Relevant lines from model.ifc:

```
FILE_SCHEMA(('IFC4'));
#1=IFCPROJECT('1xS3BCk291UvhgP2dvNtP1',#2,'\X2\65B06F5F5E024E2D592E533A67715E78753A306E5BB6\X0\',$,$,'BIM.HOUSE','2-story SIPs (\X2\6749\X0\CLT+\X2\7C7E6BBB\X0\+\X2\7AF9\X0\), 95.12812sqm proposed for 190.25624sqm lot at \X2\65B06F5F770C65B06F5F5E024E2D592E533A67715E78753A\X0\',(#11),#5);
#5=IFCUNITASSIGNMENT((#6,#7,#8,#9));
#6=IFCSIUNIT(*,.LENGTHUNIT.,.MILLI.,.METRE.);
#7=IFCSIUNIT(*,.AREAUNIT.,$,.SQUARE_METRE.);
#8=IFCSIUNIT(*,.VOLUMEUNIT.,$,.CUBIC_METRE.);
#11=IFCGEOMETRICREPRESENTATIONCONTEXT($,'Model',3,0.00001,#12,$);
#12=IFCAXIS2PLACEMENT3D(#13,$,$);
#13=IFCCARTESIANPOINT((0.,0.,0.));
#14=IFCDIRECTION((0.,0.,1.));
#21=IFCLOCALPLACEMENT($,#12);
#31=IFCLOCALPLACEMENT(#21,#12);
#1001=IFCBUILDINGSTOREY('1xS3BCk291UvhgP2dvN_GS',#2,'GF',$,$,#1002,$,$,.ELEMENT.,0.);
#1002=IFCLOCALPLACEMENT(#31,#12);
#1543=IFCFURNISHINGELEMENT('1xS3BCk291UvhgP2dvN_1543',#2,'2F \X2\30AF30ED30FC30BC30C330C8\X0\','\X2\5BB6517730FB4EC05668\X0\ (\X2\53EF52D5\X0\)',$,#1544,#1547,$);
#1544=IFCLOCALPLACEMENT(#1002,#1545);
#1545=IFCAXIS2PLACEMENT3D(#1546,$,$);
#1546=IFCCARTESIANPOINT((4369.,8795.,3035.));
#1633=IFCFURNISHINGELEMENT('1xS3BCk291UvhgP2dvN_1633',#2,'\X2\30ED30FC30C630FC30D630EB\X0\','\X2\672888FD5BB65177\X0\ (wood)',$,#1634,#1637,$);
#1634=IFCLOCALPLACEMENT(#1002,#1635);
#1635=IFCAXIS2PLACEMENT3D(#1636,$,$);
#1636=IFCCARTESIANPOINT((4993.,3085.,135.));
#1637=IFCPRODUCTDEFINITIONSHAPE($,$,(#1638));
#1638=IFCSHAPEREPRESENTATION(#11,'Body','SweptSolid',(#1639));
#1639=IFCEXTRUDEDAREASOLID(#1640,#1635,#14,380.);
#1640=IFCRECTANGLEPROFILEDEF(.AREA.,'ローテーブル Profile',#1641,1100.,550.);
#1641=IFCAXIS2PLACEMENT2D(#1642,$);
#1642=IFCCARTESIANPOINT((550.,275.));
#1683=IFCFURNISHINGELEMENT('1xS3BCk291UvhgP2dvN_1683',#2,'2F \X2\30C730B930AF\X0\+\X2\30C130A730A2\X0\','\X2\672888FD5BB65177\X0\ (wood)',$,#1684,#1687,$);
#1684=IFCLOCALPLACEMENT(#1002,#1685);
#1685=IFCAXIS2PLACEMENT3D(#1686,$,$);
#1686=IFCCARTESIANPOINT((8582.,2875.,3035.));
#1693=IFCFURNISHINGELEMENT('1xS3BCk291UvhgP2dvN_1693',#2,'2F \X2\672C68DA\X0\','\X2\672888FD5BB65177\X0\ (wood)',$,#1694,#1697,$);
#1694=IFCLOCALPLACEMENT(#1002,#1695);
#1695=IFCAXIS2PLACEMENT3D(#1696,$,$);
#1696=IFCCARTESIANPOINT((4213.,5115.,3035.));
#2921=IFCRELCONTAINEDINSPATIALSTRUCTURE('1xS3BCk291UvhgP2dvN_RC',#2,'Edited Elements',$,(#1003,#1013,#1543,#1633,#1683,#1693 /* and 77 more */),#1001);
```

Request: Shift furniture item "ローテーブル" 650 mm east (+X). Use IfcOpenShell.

```python
import ifcopenshell
import ifcopenshell.api.geometry
import ifcopenshell.util.placement

model = ifcopenshell.open("model.ifc")

item = model.by_guid("1xS3BCk291UvhgP2dvN_1633")
matrix = ifcopenshell.util.placement.get_local_placement(item.ObjectPlacement)
matrix[0, 3] += 650.0
ifcopenshell.api.geometry.edit_object_placement(model, product=item, matrix=matrix, is_si=False)

print(ifcopenshell.util.placement.get_local_placement(item.ObjectPlacement).round(3) + 0.0)

model.write("model-out.ifc")
```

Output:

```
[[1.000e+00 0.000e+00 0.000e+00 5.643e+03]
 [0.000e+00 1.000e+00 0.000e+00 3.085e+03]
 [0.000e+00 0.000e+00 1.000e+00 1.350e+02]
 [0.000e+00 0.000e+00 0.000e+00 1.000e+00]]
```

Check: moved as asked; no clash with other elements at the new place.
